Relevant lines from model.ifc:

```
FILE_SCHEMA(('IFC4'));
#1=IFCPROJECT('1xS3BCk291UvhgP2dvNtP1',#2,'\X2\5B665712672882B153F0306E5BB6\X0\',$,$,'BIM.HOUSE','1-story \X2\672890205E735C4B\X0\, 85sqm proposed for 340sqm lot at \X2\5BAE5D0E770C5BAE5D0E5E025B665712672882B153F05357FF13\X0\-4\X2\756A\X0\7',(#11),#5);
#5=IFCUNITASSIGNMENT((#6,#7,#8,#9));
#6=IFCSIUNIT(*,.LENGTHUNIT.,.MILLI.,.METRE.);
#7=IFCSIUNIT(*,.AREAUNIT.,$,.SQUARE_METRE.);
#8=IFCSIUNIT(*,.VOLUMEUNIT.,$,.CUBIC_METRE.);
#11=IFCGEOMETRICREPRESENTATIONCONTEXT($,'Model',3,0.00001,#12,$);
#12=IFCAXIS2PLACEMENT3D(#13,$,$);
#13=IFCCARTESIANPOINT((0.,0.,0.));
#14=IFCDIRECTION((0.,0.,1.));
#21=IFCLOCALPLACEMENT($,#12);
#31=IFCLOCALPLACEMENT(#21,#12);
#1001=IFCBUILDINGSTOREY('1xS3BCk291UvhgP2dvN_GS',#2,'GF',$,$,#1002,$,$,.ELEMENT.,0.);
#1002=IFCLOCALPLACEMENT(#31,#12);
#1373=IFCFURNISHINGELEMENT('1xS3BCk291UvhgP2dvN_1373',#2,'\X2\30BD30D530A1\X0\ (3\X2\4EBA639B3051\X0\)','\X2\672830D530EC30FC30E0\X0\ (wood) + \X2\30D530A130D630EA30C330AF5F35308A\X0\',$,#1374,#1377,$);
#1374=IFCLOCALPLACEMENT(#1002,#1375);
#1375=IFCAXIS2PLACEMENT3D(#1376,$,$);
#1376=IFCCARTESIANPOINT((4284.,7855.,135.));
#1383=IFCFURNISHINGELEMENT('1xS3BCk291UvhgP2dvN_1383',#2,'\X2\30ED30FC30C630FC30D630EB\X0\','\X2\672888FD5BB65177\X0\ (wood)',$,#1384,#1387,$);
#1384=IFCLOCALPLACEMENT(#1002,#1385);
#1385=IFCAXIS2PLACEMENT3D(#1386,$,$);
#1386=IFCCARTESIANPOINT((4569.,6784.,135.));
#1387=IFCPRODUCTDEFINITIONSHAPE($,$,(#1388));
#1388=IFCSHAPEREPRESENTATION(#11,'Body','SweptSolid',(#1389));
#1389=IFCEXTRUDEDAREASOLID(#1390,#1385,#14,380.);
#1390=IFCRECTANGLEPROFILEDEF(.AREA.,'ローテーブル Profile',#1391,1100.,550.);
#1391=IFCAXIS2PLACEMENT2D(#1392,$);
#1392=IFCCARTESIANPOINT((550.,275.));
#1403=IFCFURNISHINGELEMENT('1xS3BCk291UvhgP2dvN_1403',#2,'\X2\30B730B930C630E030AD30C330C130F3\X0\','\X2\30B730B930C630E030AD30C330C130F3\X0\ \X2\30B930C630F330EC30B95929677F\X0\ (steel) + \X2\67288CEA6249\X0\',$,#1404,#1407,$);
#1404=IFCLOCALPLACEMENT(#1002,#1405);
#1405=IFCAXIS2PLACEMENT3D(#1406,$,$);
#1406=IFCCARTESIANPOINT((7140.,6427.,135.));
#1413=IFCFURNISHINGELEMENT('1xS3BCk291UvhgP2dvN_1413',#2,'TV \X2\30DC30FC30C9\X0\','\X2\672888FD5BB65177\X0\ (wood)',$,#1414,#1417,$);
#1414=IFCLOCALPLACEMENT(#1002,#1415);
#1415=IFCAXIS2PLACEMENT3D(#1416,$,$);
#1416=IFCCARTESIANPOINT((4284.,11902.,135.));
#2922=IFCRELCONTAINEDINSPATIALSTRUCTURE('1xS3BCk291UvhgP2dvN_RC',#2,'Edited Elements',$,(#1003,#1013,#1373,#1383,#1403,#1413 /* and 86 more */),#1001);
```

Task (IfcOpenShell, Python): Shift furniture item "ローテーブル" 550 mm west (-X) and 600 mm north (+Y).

```python
import ifcopenshell
import ifcopenshell.api.geometry
import ifcopenshell.util.placement
import ifcopenshell.util.unit

model = ifcopenshell.open("model.ifc")
unit_scale = ifcopenshell.util.unit.calculate_unit_scale(model)

item = model.by_guid("1xS3BCk291UvhgP2dvN_1383")
matrix = ifcopenshell.util.placement.get_local_placement(item.ObjectPlacement)
matrix[0, 3] -= 0.55 / unit_scale
matrix[1, 3] += 0.6 / unit_scale
ifcopenshell.api.geometry.edit_object_placement(model, product=item, matrix=matrix, is_si=False)

print(ifcopenshell.util.placement.get_local_placement(item.ObjectPlacement).round(3) + 0.0)

model.write("model_edited.ifc")
```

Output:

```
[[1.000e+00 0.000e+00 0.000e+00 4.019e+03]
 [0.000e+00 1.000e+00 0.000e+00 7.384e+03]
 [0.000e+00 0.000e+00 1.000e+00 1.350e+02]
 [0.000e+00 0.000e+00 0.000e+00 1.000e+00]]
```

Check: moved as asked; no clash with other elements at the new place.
